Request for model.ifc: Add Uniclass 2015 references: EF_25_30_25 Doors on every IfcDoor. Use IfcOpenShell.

First a look at what the model holds.

```python
import ifcopenshell

model = ifcopenshell.open("model.ifc")
print(model.schema)
print("classifications:", [c.Name for c in model.by_type("IfcClassification")])
for ifc_class in ("IfcDoor", "IfcRoof", "IfcStair", "IfcWall", "IfcWindow"):
    print(ifc_class, len(model.by_type(ifc_class)))
```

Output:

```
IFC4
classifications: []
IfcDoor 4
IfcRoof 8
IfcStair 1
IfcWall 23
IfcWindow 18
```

```python
import ifcopenshell
import ifcopenshell.api.classification

model = ifcopenshell.open("model.ifc")

system = ifcopenshell.api.classification.add_classification(model, classification="Uniclass 2015")

codes = {
    "IfcDoor": ("EF_25_30_25", "Doors"),
}
for ifc_class, (code, name) in codes.items():
    products = model.by_type(ifc_class)
    ifcopenshell.api.classification.add_reference(
        model, products=products, classification=system, identification=code, name=name
    )
    print(code, len(products))

model.write("model-out.ifc")
```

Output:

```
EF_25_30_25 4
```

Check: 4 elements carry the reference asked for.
